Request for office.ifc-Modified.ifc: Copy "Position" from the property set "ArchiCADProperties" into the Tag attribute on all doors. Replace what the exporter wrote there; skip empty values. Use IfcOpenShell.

First a look at what the model holds.

```python
import ifcopenshell
import ifcopenshell.util.element

model = ifcopenshell.open("office.ifc-Modified.ifc")
print(model.schema)
doors = model.by_type("IfcDoor")
print(len(doors), "doors")
for e in doors[:8]:
    source = ifcopenshell.util.element.get_pset(e, "ArchiCADProperties", "Position")
    target = e.Tag
    print(e.id(), repr(source), repr(target), sep=" | ")
```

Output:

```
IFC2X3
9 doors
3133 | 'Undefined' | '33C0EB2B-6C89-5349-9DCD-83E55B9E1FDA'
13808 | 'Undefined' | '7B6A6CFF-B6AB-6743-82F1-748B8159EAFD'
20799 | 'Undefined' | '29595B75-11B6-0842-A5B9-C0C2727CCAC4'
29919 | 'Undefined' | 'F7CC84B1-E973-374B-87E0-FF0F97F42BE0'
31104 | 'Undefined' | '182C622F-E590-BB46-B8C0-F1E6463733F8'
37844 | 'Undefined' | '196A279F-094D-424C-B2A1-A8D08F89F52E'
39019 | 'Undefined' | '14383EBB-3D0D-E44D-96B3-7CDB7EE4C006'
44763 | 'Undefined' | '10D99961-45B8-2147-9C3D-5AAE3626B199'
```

```python
import ifcopenshell
import ifcopenshell.util.element

model = ifcopenshell.open("office.ifc-Modified.ifc")

count = 0
for e in model.by_type("IfcDoor"):
    value = ifcopenshell.util.element.get_pset(e, "ArchiCADProperties", "Position")
    current = e.Tag
    if not value or not value.strip() or current == value:
        continue
    e.Tag = value
    count += 1

print(count, "doors updated")

model.write("office.ifc-Modified-out.ifc")
```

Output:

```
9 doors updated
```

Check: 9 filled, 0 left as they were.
